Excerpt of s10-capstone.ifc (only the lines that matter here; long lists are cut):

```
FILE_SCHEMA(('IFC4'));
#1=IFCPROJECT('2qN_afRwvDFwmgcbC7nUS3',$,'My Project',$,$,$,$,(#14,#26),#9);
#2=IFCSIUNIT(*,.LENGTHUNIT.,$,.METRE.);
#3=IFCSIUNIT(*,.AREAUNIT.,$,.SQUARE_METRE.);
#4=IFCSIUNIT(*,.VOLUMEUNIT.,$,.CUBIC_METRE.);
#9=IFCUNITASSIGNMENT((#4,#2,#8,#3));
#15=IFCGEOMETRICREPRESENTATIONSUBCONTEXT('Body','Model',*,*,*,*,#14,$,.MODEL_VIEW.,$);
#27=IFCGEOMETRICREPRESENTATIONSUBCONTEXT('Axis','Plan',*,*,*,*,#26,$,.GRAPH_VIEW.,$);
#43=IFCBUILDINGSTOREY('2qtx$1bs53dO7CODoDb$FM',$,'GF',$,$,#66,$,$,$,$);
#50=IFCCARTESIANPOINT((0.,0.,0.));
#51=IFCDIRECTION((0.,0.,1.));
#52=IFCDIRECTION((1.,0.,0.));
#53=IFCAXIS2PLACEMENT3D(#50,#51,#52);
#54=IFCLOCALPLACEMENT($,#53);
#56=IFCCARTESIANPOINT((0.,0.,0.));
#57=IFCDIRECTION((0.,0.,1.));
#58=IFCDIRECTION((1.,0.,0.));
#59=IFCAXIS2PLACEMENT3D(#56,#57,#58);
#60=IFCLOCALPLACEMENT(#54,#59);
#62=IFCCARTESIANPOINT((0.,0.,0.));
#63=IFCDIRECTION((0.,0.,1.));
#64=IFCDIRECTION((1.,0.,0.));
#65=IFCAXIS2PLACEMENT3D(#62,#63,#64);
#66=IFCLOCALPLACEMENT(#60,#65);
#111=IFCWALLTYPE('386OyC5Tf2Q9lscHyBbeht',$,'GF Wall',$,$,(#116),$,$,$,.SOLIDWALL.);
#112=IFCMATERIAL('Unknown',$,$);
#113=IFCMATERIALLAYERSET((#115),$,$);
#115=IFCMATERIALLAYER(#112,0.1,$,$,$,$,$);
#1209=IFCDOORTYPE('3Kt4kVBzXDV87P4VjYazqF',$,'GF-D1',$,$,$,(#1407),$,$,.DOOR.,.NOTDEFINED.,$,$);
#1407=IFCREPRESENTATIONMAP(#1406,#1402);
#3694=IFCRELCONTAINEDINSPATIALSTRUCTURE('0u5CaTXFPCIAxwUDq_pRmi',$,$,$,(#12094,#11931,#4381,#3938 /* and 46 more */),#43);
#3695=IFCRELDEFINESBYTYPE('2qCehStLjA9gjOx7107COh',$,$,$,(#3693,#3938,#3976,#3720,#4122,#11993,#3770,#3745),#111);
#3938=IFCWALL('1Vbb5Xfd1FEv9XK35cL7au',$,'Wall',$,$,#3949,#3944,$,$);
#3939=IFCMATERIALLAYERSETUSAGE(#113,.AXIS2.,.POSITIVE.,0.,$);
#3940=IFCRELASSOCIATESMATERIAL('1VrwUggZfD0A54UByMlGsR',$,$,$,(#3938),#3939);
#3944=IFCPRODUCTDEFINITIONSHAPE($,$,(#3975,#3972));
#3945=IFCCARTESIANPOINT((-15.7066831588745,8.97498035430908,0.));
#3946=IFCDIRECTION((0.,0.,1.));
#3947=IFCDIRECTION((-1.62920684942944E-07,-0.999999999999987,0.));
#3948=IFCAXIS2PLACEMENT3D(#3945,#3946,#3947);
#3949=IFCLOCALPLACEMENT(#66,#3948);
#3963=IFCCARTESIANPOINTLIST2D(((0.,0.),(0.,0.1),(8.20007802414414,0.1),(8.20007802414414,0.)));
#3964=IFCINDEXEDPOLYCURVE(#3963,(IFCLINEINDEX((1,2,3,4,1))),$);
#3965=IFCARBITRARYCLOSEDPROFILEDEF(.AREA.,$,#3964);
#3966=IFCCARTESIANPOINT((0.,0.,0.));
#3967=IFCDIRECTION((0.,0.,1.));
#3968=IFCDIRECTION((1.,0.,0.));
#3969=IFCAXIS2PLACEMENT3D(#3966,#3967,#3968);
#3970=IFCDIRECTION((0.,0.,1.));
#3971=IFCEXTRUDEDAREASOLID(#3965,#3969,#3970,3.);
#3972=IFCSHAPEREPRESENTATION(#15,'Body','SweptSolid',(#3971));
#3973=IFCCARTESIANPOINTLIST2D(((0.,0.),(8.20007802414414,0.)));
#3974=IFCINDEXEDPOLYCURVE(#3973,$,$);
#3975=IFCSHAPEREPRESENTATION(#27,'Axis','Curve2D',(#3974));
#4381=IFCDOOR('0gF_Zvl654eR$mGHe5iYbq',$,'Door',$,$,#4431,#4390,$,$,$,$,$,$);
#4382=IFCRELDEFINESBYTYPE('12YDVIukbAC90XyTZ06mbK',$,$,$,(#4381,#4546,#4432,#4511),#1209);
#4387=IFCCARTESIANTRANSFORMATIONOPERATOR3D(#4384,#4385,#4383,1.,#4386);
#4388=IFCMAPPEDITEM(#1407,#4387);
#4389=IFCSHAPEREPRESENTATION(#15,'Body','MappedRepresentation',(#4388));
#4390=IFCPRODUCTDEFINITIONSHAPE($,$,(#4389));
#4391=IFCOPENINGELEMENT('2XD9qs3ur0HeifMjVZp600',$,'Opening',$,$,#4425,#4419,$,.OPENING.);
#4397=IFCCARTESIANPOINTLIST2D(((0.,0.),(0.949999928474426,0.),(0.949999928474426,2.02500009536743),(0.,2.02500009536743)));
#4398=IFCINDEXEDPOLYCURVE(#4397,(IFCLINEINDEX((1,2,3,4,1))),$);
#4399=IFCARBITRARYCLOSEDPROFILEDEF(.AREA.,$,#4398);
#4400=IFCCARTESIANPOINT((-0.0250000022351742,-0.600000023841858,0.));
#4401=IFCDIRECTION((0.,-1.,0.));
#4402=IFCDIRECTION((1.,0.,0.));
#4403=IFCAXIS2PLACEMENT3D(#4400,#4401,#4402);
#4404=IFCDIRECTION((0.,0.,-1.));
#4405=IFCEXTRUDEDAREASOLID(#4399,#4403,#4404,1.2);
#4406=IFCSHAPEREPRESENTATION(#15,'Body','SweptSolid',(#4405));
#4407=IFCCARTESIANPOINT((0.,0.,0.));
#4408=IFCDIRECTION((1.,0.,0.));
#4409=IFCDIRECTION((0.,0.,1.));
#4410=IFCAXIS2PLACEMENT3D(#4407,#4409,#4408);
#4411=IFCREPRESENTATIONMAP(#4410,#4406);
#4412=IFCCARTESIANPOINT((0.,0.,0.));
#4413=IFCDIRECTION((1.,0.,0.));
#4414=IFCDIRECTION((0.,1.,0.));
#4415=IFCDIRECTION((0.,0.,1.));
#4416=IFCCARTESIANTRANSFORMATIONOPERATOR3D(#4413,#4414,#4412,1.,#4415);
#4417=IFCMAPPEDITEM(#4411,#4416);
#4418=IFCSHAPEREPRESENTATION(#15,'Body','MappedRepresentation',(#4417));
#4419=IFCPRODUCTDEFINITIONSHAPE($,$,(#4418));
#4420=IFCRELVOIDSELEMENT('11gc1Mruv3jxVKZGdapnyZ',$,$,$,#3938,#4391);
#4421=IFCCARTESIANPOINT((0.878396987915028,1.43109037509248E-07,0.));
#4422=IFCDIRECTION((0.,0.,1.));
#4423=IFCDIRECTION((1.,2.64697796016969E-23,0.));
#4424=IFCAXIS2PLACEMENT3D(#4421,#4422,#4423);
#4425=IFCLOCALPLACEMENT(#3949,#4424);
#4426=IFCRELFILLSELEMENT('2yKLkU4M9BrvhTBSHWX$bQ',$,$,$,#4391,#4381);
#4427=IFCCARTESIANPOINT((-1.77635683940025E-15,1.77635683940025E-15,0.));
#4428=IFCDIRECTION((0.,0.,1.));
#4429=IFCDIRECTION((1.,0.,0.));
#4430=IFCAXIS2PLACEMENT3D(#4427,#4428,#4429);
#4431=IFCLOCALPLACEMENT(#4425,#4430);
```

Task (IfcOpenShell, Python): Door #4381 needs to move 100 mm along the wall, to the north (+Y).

```python
import ifcopenshell
import ifcopenshell.api.geometry
import ifcopenshell.util.placement

model = ifcopenshell.open("s10-capstone.ifc")

door = model.by_guid("0gF_Zvl654eR$mGHe5iYbq")
opening = door.FillsVoids[0].RelatingOpeningElement
wall = opening.VoidsElements[0].RelatingBuildingElement

wall_matrix = ifcopenshell.util.placement.get_local_placement(wall.ObjectPlacement)
shift = wall_matrix[:3, 0] * -0.1
before = ifcopenshell.util.placement.get_local_placement(door.ObjectPlacement)[:3, 3].copy()

# The door is placed relative to its opening, so it follows when the opening moves.
matrix = ifcopenshell.util.placement.get_local_placement(opening.ObjectPlacement)
matrix[:3, 3] += shift
ifcopenshell.api.geometry.edit_object_placement(
    model, product=opening, matrix=matrix, is_si=False, should_transform_children=True
)

after = ifcopenshell.util.placement.get_local_placement(door.ObjectPlacement)[:3, 3]
print("door moved by", (after - before).round(3) + 0.0)

model.write("s10-capstone_updated.ifc")
```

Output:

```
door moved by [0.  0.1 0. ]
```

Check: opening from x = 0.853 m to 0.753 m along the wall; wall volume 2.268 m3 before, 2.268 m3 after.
